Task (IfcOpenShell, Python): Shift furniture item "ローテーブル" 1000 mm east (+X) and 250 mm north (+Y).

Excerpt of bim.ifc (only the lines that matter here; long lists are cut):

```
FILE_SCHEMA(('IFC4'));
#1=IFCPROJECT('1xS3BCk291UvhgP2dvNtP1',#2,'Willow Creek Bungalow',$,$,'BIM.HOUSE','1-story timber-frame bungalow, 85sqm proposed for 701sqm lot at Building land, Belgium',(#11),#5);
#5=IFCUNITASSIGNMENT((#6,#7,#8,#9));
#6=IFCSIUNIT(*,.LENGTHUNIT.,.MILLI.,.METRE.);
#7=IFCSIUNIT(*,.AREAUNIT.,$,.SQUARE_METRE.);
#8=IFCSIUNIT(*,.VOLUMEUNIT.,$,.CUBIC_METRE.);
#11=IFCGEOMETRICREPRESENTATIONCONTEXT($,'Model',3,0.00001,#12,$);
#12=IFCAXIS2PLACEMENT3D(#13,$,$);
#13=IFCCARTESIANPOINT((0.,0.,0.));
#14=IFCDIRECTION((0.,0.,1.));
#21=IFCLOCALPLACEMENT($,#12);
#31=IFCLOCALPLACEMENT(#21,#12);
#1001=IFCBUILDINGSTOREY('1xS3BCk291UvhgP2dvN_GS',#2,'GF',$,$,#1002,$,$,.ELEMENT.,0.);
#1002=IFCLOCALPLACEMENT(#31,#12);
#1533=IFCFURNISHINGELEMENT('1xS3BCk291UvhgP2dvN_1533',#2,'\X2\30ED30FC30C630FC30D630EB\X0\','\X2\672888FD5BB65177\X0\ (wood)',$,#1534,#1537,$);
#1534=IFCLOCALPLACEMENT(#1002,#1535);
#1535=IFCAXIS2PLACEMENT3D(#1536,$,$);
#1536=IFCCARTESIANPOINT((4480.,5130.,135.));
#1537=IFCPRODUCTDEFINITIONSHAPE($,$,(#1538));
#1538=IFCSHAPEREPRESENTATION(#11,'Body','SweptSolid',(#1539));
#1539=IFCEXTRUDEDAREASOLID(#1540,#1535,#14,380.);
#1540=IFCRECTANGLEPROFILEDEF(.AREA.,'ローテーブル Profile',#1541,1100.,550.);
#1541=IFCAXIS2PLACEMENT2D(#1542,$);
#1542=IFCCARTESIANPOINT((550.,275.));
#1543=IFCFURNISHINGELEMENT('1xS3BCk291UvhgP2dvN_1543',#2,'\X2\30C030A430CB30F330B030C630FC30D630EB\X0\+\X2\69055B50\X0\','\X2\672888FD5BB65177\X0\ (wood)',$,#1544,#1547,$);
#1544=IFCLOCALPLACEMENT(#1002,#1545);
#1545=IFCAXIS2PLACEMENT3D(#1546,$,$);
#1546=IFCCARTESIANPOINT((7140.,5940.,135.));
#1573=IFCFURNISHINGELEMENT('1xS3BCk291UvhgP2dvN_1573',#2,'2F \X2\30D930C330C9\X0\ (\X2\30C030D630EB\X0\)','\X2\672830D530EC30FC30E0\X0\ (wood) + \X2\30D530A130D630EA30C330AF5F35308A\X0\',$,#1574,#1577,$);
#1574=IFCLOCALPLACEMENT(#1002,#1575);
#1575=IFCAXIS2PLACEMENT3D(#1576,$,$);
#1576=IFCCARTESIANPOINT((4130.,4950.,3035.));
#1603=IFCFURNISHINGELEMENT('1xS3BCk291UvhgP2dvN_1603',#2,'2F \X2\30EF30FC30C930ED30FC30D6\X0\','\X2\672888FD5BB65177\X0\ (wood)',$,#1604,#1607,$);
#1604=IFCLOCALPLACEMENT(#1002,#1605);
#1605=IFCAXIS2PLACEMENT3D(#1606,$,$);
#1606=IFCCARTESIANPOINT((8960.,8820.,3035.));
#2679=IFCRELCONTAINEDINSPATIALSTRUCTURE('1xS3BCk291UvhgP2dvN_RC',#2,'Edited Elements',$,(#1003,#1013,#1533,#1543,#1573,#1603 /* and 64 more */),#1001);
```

```python
import ifcopenshell
import ifcopenshell.api.geometry
import ifcopenshell.util.placement
import ifcopenshell.util.unit

model = ifcopenshell.open("bim.ifc")
unit_scale = ifcopenshell.util.unit.calculate_unit_scale(model)

item = model.by_id(1533)
matrix = ifcopenshell.util.placement.get_local_placement(item.ObjectPlacement)
matrix[0, 3] += 1 / unit_scale
matrix[1, 3] += 0.25 / unit_scale
ifcopenshell.api.geometry.edit_object_placement(model, product=item, matrix=matrix, is_si=False)

print(ifcopenshell.util.placement.get_local_placement(item.ObjectPlacement).round(3) + 0.0)

model.write("bim-out.ifc")
```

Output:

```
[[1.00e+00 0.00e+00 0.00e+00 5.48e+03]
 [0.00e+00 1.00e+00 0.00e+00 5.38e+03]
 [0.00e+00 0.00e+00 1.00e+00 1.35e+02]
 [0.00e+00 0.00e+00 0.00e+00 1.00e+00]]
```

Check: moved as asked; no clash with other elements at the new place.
